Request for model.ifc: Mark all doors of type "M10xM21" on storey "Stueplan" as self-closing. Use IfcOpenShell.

First a look at what the model holds.

```python
import ifcopenshell
import ifcopenshell.util.element

model = ifcopenshell.open("model.ifc")
print(model.schema)
storey = next(s for s in model.by_type("IfcBuildingStorey") if s.Name == "Stueplan")
doors = [e for e in ifcopenshell.util.element.get_decomposition(storey) if e.is_a("IfcDoor")]
seen = {}
for e in doors:
    element_type = ifcopenshell.util.element.get_type(e)
    key = (element_type.Name if element_type != e and element_type else None, ifcopenshell.util.element.get_pset(e, "Pset_DoorCommon", "SelfClosing"))
    seen[key] = seen.get(key, 0) + 1
for (name, value), count in sorted(seen.items(), key=str):
    print(count, "x", name, "|", value)
```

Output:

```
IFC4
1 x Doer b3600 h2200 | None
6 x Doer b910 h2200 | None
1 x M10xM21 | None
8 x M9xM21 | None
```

```python
import ifcopenshell
import ifcopenshell.api.pset
import ifcopenshell.util.element

model = ifcopenshell.open("model.ifc")

storey = next(s for s in model.by_type("IfcBuildingStorey") if s.Name == "Stueplan")
doors = [e for e in ifcopenshell.util.element.get_decomposition(storey) if e.is_a("IfcDoor")]

count = 0
for e in doors:
    element_type = ifcopenshell.util.element.get_type(e)
    if element_type in (None, e) or element_type.Name != "M10xM21":
        continue
    # add_pset returns the element's existing set when there is one.
    pset = ifcopenshell.api.pset.add_pset(model, product=e, name="Pset_DoorCommon")
    ifcopenshell.api.pset.edit_pset(model, pset=pset, properties={"SelfClosing": True})
    count += 1

print(count, "doors updated")

model.write("model_updated.ifc")
```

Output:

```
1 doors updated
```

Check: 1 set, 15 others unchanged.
